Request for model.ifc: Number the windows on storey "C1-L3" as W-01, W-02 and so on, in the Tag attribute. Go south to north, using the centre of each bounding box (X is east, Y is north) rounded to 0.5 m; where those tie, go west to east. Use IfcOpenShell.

First a look at what the model holds.

```python
import ifcopenshell
import ifcopenshell.util.element
import ifcopenshell.util.placement

model = ifcopenshell.open("model.ifc")
print(model.schema)
storey = next(s for s in model.by_type("IfcBuildingStorey") if s.Name == "C1-L3")
windows = [e for e in ifcopenshell.util.element.get_decomposition(storey) if e.is_a("IfcWindow")]
for e in sorted(windows, key=lambda e: e.id()):
    origin = ifcopenshell.util.placement.get_local_placement(e.ObjectPlacement)[:3, 3]
    print(e.id(), e.Tag, e.Name, origin.round(2) + 0.0, sep=" | ")
```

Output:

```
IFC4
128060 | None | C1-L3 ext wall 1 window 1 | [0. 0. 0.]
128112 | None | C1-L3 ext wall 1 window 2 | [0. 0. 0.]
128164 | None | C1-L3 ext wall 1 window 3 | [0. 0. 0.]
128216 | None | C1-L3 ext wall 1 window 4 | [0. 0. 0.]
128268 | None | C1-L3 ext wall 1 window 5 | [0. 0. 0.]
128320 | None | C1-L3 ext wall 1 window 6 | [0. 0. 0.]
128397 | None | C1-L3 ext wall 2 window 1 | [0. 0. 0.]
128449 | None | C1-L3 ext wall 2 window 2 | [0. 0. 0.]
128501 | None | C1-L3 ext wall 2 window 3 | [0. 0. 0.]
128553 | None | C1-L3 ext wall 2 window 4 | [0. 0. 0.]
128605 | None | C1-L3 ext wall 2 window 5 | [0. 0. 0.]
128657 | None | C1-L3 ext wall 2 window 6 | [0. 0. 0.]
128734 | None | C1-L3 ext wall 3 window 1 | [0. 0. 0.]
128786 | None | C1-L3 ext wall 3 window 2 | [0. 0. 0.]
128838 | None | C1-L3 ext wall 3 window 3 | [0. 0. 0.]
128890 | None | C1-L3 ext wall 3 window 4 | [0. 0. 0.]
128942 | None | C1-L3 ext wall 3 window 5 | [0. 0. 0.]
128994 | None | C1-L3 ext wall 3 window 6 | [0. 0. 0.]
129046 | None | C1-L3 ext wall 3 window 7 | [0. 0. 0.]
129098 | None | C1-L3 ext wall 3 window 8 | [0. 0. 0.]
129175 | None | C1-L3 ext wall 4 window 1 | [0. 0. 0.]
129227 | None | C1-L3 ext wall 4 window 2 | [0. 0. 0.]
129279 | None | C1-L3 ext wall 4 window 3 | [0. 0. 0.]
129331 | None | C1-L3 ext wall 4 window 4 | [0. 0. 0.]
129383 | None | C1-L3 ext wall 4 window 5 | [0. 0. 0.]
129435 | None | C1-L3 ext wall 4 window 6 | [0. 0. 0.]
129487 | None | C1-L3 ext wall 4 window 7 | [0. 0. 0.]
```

```python
import ifcopenshell
import ifcopenshell.geom
import ifcopenshell.util.element
import ifcopenshell.util.shape

model = ifcopenshell.open("model.ifc")
settings = ifcopenshell.geom.settings()
settings.set("use-world-coords", True)


def centre(element):
    shape = ifcopenshell.geom.create_shape(settings, element)
    return ifcopenshell.util.shape.get_bbox_centroid(shape.geometry)


storey = next(s for s in model.by_type("IfcBuildingStorey") if s.Name == "C1-L3")
windows = [e for e in ifcopenshell.util.element.get_decomposition(storey) if e.is_a("IfcWindow")]

# Insertion points can sit at a corner or the storey origin, so sort by the geometry (in metres).
centres = {e: centre(e) for e in windows}
windows.sort(key=lambda e: (round(centres[e][1] / 0.5), centres[e][0]))

for i, e in enumerate(windows, start=1):
    number = f"W-{i:02d}"
    e.Tag = number
    print(e.id(), number)

model.write("model_updated.ifc")
```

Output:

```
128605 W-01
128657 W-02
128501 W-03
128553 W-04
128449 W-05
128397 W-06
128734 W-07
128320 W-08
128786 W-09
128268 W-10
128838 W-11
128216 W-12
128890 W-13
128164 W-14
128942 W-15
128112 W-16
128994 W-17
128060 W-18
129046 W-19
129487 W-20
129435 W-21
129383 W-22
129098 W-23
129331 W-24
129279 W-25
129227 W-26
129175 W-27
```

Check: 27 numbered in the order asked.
